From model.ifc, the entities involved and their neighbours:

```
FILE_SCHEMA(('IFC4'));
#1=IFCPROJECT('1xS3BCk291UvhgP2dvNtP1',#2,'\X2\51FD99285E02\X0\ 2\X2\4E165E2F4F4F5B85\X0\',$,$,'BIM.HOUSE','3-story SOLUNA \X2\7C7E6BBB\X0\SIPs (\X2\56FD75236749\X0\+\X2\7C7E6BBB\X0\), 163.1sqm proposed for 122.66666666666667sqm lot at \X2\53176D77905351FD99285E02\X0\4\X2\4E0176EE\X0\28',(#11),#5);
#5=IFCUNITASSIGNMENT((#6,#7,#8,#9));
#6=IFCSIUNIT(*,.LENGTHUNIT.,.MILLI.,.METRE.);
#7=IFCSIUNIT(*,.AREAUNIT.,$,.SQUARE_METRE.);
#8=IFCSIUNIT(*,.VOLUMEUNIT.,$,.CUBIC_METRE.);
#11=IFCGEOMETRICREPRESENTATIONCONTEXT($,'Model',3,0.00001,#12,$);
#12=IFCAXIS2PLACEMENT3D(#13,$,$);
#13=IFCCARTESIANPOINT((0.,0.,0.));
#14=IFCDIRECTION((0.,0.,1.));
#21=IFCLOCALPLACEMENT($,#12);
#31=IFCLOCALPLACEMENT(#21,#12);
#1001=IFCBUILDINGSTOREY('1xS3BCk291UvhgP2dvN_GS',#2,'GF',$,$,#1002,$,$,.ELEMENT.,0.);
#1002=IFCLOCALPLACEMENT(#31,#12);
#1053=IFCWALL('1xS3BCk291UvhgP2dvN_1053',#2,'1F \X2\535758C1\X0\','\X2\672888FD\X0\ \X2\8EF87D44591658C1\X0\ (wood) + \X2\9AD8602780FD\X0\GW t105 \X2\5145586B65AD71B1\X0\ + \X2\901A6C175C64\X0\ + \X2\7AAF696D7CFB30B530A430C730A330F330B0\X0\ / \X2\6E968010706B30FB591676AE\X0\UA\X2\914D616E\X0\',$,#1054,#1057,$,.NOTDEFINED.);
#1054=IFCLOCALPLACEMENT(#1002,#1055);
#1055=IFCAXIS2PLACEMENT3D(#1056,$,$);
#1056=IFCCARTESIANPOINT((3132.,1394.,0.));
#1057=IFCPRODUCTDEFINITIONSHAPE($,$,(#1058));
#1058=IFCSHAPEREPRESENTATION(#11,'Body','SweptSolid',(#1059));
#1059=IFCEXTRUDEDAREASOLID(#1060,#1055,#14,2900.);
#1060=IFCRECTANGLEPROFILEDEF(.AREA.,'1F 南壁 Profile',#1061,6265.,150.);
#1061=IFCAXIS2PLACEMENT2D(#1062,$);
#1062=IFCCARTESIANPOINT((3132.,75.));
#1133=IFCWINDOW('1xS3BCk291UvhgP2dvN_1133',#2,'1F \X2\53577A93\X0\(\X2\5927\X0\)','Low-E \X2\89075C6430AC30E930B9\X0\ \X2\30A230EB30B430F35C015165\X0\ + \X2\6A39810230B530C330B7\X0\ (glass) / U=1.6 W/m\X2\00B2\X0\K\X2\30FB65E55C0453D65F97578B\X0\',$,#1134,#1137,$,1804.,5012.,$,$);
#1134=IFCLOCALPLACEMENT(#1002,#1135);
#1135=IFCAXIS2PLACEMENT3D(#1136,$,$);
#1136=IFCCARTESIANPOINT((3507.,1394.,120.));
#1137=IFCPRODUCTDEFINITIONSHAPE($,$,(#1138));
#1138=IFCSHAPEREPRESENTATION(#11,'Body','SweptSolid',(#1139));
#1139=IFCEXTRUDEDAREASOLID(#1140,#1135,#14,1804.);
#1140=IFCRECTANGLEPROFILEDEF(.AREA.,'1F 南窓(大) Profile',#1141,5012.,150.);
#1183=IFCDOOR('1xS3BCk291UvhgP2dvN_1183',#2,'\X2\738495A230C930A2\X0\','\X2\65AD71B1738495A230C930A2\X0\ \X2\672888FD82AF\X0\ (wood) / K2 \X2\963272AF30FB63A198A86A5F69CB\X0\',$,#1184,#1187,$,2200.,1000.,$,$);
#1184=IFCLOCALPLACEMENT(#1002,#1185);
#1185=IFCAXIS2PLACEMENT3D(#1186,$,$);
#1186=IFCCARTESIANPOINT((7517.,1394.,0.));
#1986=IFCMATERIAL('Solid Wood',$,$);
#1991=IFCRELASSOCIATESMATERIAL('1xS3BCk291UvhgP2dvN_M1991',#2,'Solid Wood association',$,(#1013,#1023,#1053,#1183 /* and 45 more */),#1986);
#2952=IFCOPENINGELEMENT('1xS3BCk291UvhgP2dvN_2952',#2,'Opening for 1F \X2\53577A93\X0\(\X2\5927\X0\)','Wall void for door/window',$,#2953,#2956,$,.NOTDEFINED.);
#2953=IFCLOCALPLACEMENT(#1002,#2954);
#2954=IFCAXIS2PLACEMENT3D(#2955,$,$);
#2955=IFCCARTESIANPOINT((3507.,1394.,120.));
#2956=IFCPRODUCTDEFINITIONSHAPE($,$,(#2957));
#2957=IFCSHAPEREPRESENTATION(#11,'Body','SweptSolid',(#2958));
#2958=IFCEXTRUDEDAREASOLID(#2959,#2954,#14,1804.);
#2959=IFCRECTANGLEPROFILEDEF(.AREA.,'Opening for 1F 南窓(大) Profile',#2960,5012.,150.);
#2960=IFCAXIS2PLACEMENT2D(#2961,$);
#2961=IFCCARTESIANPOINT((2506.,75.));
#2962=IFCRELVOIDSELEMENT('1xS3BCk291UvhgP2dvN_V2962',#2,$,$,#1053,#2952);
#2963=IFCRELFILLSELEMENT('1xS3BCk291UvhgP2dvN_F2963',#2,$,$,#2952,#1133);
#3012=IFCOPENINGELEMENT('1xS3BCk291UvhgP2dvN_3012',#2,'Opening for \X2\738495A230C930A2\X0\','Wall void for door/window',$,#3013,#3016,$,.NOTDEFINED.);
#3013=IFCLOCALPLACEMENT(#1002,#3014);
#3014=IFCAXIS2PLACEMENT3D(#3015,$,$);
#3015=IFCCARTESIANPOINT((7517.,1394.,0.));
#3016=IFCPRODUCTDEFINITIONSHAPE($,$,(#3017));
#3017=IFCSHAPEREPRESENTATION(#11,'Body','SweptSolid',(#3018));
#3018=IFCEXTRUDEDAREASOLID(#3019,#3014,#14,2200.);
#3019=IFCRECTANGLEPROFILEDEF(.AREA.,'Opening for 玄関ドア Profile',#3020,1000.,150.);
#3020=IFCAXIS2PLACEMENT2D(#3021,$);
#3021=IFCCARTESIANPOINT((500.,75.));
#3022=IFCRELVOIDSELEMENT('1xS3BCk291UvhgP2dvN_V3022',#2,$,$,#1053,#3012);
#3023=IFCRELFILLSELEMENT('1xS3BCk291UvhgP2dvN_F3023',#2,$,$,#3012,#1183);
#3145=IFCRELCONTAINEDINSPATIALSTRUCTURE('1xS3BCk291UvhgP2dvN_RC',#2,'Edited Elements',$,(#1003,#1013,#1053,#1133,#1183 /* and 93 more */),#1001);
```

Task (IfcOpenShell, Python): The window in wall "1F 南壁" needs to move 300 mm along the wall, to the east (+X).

```python
import ifcopenshell
import ifcopenshell.api.geometry
import ifcopenshell.util.placement
import ifcopenshell.util.unit

model = ifcopenshell.open("model.ifc")
unit_scale = ifcopenshell.util.unit.calculate_unit_scale(model)

window = model.by_guid("1xS3BCk291UvhgP2dvN_1133")
opening = window.FillsVoids[0].RelatingOpeningElement
wall = opening.VoidsElements[0].RelatingBuildingElement

wall_matrix = ifcopenshell.util.placement.get_local_placement(wall.ObjectPlacement)
shift = wall_matrix[:3, 0] * 0.3 / unit_scale
before = ifcopenshell.util.placement.get_local_placement(window.ObjectPlacement)[:3, 3].copy()

# The window is not placed relative to its opening, so move both.
for product in (opening, window):
    matrix = ifcopenshell.util.placement.get_local_placement(product.ObjectPlacement)
    matrix[:3, 3] += shift
    ifcopenshell.api.geometry.edit_object_placement(model, product=product, matrix=matrix, is_si=False)

after = ifcopenshell.util.placement.get_local_placement(window.ObjectPlacement)[:3, 3]
print("window moved by", (after - before).round(3) + 0.0)

model.write("model_rev.ifc")
```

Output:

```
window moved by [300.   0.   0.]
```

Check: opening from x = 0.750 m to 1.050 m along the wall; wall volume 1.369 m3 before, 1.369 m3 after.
